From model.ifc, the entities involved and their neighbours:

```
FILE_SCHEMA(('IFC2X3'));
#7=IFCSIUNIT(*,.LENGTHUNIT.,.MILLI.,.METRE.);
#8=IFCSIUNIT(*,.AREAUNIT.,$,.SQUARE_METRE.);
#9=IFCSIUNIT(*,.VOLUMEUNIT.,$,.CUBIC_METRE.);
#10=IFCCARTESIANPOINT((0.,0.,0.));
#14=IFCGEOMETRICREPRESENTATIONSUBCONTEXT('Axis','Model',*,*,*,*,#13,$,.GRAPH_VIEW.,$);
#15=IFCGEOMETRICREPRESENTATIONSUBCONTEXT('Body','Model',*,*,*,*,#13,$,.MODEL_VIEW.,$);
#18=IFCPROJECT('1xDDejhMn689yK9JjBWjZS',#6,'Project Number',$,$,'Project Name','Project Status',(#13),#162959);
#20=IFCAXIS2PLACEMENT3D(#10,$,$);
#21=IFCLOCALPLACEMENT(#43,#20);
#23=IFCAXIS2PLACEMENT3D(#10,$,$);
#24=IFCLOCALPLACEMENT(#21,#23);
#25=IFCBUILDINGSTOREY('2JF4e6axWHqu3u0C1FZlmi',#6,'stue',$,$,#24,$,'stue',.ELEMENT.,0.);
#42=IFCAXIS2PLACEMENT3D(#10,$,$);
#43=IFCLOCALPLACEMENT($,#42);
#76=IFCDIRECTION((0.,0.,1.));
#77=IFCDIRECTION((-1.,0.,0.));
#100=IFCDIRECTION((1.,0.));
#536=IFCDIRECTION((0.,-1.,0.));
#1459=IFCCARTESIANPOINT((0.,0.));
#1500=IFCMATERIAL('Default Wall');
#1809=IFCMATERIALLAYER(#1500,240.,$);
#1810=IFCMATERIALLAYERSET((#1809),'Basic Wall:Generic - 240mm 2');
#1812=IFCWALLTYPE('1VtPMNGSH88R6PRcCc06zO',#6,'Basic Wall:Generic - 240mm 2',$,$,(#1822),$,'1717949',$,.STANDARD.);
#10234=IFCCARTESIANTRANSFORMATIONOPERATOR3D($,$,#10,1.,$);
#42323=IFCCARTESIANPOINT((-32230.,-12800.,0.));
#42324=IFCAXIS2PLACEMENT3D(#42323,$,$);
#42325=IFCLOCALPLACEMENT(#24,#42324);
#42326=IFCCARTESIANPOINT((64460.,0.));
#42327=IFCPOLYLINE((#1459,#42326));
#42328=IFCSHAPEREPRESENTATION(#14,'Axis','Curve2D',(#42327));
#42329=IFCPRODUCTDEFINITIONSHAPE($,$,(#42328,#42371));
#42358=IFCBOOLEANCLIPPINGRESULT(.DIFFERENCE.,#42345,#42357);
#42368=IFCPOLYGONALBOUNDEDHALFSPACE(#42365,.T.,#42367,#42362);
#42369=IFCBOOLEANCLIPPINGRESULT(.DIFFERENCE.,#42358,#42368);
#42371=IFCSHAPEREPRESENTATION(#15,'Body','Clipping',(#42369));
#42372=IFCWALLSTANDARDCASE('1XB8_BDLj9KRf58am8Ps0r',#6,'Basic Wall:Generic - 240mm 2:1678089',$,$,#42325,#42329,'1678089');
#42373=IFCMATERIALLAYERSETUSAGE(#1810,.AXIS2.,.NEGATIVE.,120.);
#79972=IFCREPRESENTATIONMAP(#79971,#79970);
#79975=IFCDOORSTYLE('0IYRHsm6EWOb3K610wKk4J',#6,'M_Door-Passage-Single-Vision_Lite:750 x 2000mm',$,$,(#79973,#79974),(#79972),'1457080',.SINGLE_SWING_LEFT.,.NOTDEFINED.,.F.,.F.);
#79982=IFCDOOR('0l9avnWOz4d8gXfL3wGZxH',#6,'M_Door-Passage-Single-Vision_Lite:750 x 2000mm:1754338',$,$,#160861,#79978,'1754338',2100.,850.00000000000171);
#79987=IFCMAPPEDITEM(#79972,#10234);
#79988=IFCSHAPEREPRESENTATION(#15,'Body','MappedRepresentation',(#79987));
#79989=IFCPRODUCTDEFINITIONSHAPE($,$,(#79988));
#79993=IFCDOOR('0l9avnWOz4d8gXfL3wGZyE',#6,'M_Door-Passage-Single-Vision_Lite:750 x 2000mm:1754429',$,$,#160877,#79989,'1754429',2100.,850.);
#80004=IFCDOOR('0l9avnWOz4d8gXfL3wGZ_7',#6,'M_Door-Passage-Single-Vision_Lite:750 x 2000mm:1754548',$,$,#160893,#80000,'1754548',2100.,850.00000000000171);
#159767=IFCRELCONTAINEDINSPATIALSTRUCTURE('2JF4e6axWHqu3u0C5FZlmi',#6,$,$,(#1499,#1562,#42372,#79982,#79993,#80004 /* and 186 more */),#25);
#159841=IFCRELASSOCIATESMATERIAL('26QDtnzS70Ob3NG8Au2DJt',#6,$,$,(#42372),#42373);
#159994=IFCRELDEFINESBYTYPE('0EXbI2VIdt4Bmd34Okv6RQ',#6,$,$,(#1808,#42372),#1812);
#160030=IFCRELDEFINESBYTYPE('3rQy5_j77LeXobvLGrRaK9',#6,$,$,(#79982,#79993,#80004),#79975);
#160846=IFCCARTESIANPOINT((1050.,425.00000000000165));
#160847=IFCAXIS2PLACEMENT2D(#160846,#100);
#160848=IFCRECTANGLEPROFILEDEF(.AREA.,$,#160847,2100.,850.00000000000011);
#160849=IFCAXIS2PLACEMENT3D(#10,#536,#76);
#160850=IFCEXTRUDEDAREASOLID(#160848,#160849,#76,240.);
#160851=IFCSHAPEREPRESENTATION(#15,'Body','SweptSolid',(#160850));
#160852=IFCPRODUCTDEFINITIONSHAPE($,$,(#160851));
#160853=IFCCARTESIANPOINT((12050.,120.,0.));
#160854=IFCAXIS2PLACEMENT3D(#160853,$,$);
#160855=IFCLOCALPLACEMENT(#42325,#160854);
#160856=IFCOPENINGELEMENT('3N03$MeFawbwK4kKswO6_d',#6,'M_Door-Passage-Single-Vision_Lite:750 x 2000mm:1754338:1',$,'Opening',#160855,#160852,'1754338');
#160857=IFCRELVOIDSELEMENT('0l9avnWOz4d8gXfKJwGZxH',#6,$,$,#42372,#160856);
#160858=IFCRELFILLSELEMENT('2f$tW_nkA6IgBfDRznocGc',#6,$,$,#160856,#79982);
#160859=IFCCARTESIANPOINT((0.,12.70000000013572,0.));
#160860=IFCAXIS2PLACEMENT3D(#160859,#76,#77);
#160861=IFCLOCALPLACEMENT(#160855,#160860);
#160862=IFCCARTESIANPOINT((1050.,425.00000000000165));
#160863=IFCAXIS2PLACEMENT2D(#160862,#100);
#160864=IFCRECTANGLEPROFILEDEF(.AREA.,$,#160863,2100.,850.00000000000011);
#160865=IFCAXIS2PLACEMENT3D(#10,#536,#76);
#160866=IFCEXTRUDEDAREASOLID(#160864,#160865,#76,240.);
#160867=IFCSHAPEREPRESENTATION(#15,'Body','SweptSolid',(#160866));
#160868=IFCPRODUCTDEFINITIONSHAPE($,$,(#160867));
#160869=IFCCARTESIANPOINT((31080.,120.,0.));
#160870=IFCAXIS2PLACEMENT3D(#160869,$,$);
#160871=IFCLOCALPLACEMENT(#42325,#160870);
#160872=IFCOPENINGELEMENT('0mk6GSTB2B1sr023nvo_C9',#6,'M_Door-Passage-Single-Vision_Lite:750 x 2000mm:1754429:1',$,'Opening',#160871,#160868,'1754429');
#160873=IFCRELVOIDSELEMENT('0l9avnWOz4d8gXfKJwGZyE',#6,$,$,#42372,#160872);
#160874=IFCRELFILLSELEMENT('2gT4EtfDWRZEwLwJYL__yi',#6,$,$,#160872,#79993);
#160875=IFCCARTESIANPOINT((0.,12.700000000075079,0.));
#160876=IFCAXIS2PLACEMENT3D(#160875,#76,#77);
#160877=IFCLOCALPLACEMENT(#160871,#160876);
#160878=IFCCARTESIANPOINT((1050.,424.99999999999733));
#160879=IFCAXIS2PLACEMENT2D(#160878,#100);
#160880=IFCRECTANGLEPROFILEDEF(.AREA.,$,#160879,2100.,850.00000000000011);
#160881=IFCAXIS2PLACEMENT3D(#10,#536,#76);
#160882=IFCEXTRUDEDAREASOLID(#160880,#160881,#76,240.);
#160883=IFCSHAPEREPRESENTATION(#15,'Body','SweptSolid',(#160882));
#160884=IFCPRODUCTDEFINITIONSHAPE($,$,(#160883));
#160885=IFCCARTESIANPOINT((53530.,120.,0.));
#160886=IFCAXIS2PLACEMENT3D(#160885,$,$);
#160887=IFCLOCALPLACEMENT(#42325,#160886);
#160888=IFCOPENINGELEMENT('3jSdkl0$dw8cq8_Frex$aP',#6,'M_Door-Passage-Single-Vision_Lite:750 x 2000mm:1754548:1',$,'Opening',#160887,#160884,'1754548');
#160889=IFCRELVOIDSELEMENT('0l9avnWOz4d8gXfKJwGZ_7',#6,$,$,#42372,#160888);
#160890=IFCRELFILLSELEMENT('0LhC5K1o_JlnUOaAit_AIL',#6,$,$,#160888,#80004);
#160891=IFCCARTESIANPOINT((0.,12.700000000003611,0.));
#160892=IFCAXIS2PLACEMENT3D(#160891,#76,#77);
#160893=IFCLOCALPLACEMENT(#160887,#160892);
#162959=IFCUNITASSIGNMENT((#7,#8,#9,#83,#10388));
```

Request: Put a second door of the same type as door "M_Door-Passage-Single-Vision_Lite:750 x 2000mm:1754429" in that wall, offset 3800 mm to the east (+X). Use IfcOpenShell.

```python
import ifcopenshell
import ifcopenshell.api.feature
import ifcopenshell.api.geometry
import ifcopenshell.api.root
import ifcopenshell.geom
import ifcopenshell.util.element
import ifcopenshell.util.placement
import ifcopenshell.util.shape
import ifcopenshell.util.unit

model = ifcopenshell.open("model.ifc")
unit_scale = ifcopenshell.util.unit.calculate_unit_scale(model)
settings = ifcopenshell.geom.settings()


def volume(element):
    """Net volume in cubic metres, openings subtracted."""
    shape = ifcopenshell.geom.create_shape(settings, element)
    return ifcopenshell.util.shape.get_volume(shape.geometry)


def reuse_history(source, copy):
    """copy_class also copies each property set's owner history, people and application; keep the originals."""
    for rel in copy.IsDefinedBy:
        if rel.is_a("IfcRelDefinesByProperties") and (history := rel.RelatingPropertyDefinition.OwnerHistory):
            rel.RelatingPropertyDefinition.OwnerHistory = source.OwnerHistory
            ifcopenshell.util.element.remove_deep2(model, history)


door = model.by_id(79993)
opening = door.FillsVoids[0].RelatingOpeningElement
wall = opening.VoidsElements[0].RelatingBuildingElement
before = volume(wall)
shift = ifcopenshell.util.placement.get_local_placement(wall.ObjectPlacement)[:3, 0] * 3.8 / unit_scale

# copy_class copies the void relationship, type, container and properties, but no geometry.
new_opening = ifcopenshell.api.root.copy_class(model, product=opening)
new_opening.Representation = ifcopenshell.util.element.copy_deep(
    model, opening.Representation, exclude=["IfcGeometricRepresentationContext", "IfcRepresentationMap"]
)
new_opening.Name = "M_Door-Passage-Single-Vision_Lite:750 x 2000mm"
new_opening.Tag = None
new_door = ifcopenshell.api.root.copy_class(model, product=door)
new_door.Representation = ifcopenshell.util.element.copy_deep(
    model, door.Representation, exclude=["IfcGeometricRepresentationContext", "IfcRepresentationMap"]
)
new_door.Name = "M_Door-Passage-Single-Vision_Lite:750 x 2000mm"
new_door.Tag = None
reuse_history(door, new_door)
fills = ifcopenshell.api.feature.add_filling(model, opening=new_opening, element=new_door)
fills.OwnerHistory = new_door.OwnerHistory  # required in IFC2X3

for old, new in ((opening, new_opening), (door, new_door)):
    matrix = ifcopenshell.util.placement.get_local_placement(old.ObjectPlacement)
    matrix[:3, 3] += shift
    ifcopenshell.api.geometry.edit_object_placement(model, product=new, matrix=matrix, is_si=False)

after = volume(wall)

print(f"wall volume {before:.3f} -> {after:.3f} m3")

model.write("model-out.ifc")
```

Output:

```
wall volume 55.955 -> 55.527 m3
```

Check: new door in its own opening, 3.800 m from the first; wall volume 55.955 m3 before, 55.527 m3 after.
